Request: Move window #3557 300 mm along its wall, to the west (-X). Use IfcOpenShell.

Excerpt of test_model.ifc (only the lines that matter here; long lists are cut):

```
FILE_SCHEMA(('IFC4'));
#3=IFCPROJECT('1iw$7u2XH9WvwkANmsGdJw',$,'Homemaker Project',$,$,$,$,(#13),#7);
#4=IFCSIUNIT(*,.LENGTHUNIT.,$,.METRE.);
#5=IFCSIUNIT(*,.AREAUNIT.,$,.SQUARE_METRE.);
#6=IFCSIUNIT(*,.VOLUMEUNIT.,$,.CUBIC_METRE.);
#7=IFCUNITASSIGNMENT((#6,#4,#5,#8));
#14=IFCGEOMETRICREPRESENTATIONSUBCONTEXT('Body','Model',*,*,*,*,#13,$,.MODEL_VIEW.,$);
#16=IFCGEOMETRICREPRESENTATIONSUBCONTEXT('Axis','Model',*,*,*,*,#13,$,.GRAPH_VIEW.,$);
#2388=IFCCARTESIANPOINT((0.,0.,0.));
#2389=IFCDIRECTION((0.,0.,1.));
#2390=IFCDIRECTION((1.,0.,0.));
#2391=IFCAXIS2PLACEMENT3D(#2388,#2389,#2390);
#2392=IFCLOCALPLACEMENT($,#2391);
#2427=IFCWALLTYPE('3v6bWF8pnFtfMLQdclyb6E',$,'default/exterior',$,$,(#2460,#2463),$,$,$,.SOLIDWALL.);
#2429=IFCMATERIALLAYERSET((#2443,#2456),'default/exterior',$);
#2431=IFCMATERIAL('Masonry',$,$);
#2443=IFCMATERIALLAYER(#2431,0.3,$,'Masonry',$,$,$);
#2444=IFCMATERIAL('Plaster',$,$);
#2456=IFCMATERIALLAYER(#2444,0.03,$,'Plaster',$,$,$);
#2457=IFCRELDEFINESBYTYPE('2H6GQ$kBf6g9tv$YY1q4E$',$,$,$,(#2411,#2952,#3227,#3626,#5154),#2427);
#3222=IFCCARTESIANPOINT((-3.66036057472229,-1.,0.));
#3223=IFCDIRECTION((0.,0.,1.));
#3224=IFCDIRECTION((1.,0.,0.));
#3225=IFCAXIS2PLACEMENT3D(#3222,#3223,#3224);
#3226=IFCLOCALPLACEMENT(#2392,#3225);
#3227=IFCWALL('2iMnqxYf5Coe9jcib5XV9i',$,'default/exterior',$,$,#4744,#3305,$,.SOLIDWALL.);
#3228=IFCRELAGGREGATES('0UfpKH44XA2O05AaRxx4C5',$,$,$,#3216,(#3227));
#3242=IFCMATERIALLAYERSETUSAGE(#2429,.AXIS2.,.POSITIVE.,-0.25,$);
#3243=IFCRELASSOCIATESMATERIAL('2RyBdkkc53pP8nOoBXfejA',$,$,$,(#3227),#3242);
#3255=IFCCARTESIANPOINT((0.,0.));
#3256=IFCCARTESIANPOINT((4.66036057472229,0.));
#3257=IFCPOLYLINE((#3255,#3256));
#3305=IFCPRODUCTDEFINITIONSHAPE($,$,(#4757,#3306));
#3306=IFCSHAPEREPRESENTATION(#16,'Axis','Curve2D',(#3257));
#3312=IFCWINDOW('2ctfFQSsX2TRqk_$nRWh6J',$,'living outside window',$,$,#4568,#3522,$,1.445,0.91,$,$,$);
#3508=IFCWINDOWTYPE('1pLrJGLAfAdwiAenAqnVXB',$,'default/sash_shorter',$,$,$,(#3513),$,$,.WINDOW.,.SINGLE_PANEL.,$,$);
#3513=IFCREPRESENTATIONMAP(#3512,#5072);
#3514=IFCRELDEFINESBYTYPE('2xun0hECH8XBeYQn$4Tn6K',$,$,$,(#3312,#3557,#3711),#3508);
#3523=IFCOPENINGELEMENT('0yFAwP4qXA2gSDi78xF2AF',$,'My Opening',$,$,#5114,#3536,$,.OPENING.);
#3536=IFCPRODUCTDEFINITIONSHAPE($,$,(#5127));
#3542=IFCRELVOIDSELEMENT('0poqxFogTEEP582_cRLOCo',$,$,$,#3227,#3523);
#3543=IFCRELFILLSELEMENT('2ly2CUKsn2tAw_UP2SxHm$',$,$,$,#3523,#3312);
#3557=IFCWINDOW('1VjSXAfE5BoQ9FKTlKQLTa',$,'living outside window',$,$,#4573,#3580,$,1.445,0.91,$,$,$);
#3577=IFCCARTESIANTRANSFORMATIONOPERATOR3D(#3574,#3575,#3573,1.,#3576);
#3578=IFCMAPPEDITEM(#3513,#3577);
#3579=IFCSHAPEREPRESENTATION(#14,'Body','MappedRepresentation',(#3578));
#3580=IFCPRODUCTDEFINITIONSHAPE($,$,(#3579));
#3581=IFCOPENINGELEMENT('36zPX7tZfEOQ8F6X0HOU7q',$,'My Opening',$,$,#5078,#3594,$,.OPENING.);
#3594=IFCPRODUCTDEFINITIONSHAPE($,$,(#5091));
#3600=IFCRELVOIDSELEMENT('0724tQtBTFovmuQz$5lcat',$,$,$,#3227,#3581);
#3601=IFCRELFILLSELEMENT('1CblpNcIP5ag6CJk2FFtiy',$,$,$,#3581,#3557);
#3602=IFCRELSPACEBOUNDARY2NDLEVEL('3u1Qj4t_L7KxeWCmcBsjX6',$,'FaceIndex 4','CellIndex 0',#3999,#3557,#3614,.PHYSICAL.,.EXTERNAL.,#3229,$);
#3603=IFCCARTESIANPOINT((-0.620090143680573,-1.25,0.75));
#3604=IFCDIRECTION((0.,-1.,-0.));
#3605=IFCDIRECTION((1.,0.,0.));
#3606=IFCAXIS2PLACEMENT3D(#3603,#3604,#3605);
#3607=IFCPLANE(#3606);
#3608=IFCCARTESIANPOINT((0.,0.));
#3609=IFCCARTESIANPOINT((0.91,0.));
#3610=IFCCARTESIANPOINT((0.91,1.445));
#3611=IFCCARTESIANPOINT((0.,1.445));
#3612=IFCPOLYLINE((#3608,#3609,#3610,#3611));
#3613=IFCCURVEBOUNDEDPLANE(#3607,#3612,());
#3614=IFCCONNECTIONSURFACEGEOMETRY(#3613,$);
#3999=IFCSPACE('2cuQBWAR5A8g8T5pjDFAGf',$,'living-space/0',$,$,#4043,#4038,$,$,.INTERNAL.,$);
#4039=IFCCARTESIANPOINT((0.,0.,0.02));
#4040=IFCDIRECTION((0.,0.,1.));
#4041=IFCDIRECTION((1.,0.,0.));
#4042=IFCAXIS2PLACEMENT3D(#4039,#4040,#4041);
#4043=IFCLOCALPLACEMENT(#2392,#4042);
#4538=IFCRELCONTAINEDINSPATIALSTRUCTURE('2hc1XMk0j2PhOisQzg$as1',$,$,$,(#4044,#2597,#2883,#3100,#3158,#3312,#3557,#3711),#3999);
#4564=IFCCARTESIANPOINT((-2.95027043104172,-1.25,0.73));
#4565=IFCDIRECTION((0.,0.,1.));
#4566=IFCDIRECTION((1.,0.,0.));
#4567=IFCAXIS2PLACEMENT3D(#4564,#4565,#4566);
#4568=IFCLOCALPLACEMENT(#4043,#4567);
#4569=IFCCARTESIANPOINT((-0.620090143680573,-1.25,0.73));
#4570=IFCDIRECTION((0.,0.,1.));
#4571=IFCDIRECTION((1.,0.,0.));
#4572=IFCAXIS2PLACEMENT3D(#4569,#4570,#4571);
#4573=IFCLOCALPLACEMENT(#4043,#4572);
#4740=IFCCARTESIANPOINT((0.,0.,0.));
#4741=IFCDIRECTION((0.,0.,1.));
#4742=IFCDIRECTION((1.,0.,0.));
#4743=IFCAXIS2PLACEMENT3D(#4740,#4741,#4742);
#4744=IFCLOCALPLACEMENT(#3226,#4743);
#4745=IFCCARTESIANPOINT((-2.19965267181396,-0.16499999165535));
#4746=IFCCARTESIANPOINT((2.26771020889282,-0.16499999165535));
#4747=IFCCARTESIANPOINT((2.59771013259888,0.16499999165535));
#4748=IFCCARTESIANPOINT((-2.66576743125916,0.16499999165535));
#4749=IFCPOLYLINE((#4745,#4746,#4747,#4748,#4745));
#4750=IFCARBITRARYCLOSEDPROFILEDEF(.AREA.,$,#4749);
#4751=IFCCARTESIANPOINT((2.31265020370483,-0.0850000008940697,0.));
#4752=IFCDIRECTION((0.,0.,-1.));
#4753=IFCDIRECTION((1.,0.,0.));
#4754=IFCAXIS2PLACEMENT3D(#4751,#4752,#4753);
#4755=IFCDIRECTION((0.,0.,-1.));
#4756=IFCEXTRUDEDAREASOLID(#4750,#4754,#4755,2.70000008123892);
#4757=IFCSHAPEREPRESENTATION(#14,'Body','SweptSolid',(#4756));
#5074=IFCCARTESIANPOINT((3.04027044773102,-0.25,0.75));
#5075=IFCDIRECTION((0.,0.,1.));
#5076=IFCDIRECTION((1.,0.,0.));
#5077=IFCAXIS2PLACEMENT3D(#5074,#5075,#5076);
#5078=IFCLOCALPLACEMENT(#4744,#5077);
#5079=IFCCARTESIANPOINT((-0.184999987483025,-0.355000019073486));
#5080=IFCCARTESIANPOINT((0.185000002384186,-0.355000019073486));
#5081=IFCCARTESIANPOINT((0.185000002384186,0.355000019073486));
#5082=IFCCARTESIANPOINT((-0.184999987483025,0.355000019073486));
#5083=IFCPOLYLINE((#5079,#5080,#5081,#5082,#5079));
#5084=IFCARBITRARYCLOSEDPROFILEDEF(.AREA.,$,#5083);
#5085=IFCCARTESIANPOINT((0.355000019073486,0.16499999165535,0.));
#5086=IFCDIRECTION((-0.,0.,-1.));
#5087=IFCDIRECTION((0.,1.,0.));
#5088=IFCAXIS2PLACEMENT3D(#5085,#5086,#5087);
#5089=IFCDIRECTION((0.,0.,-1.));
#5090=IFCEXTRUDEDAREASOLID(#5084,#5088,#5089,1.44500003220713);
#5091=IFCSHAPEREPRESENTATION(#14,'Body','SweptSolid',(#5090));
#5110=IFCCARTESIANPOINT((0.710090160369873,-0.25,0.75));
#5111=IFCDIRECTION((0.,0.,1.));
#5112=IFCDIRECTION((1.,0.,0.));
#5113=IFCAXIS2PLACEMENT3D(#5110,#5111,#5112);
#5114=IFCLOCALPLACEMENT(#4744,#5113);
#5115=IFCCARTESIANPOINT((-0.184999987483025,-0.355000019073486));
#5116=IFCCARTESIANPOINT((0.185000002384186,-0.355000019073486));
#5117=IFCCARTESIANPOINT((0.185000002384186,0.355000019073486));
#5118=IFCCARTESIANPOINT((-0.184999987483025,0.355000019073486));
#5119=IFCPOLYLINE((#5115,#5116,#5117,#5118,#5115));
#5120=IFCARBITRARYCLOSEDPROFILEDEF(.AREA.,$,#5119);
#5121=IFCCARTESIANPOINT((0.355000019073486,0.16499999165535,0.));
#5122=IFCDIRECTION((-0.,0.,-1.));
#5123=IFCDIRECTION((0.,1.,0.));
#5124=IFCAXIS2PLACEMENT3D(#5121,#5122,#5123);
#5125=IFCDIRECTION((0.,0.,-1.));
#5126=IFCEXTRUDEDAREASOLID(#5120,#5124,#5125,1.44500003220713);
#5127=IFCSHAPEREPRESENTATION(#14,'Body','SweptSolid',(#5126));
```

```python
import numpy as np
import ifcopenshell
import ifcopenshell.api.geometry
import ifcopenshell.util.placement

model = ifcopenshell.open("test_model.ifc")

window = model.by_guid("1VjSXAfE5BoQ9FKTlKQLTa")
opening = window.FillsVoids[0].RelatingOpeningElement
wall = opening.VoidsElements[0].RelatingBuildingElement

wall_matrix = ifcopenshell.util.placement.get_local_placement(wall.ObjectPlacement)
shift = wall_matrix[:3, 0] * -0.3
before = ifcopenshell.util.placement.get_local_placement(window.ObjectPlacement)[:3, 3].copy()

# The window is not placed relative to its opening, so move both.
for product in (opening, window):
    matrix = ifcopenshell.util.placement.get_local_placement(product.ObjectPlacement)
    matrix[:3, 3] += shift
    ifcopenshell.api.geometry.edit_object_placement(model, product=product, matrix=matrix, is_si=False)

# Space boundary surfaces are stored in each space's coordinates; move them too.
for rel in window.ProvidesBoundaries:
    if not rel.ConnectionGeometry:
        continue
    surface = rel.ConnectionGeometry.SurfaceOnRelatingElement.BasisSurface
    space_matrix = ifcopenshell.util.placement.get_local_placement(rel.RelatingSpace.ObjectPlacement)
    point = np.array(surface.Position.Location.Coordinates) + space_matrix[:3, :3].T @ shift
    surface.Position = model.createIfcAxis2Placement3D(
        model.createIfcCartesianPoint(point.tolist()), surface.Position.Axis, surface.Position.RefDirection
    )

after = ifcopenshell.util.placement.get_local_placement(window.ObjectPlacement)[:3, 3]
print("window moved by", (after - before).round(3) + 0.0)

model.write("test_model-out.ifc")
```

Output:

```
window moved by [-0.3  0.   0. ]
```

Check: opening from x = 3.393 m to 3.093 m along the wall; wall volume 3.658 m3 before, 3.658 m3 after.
